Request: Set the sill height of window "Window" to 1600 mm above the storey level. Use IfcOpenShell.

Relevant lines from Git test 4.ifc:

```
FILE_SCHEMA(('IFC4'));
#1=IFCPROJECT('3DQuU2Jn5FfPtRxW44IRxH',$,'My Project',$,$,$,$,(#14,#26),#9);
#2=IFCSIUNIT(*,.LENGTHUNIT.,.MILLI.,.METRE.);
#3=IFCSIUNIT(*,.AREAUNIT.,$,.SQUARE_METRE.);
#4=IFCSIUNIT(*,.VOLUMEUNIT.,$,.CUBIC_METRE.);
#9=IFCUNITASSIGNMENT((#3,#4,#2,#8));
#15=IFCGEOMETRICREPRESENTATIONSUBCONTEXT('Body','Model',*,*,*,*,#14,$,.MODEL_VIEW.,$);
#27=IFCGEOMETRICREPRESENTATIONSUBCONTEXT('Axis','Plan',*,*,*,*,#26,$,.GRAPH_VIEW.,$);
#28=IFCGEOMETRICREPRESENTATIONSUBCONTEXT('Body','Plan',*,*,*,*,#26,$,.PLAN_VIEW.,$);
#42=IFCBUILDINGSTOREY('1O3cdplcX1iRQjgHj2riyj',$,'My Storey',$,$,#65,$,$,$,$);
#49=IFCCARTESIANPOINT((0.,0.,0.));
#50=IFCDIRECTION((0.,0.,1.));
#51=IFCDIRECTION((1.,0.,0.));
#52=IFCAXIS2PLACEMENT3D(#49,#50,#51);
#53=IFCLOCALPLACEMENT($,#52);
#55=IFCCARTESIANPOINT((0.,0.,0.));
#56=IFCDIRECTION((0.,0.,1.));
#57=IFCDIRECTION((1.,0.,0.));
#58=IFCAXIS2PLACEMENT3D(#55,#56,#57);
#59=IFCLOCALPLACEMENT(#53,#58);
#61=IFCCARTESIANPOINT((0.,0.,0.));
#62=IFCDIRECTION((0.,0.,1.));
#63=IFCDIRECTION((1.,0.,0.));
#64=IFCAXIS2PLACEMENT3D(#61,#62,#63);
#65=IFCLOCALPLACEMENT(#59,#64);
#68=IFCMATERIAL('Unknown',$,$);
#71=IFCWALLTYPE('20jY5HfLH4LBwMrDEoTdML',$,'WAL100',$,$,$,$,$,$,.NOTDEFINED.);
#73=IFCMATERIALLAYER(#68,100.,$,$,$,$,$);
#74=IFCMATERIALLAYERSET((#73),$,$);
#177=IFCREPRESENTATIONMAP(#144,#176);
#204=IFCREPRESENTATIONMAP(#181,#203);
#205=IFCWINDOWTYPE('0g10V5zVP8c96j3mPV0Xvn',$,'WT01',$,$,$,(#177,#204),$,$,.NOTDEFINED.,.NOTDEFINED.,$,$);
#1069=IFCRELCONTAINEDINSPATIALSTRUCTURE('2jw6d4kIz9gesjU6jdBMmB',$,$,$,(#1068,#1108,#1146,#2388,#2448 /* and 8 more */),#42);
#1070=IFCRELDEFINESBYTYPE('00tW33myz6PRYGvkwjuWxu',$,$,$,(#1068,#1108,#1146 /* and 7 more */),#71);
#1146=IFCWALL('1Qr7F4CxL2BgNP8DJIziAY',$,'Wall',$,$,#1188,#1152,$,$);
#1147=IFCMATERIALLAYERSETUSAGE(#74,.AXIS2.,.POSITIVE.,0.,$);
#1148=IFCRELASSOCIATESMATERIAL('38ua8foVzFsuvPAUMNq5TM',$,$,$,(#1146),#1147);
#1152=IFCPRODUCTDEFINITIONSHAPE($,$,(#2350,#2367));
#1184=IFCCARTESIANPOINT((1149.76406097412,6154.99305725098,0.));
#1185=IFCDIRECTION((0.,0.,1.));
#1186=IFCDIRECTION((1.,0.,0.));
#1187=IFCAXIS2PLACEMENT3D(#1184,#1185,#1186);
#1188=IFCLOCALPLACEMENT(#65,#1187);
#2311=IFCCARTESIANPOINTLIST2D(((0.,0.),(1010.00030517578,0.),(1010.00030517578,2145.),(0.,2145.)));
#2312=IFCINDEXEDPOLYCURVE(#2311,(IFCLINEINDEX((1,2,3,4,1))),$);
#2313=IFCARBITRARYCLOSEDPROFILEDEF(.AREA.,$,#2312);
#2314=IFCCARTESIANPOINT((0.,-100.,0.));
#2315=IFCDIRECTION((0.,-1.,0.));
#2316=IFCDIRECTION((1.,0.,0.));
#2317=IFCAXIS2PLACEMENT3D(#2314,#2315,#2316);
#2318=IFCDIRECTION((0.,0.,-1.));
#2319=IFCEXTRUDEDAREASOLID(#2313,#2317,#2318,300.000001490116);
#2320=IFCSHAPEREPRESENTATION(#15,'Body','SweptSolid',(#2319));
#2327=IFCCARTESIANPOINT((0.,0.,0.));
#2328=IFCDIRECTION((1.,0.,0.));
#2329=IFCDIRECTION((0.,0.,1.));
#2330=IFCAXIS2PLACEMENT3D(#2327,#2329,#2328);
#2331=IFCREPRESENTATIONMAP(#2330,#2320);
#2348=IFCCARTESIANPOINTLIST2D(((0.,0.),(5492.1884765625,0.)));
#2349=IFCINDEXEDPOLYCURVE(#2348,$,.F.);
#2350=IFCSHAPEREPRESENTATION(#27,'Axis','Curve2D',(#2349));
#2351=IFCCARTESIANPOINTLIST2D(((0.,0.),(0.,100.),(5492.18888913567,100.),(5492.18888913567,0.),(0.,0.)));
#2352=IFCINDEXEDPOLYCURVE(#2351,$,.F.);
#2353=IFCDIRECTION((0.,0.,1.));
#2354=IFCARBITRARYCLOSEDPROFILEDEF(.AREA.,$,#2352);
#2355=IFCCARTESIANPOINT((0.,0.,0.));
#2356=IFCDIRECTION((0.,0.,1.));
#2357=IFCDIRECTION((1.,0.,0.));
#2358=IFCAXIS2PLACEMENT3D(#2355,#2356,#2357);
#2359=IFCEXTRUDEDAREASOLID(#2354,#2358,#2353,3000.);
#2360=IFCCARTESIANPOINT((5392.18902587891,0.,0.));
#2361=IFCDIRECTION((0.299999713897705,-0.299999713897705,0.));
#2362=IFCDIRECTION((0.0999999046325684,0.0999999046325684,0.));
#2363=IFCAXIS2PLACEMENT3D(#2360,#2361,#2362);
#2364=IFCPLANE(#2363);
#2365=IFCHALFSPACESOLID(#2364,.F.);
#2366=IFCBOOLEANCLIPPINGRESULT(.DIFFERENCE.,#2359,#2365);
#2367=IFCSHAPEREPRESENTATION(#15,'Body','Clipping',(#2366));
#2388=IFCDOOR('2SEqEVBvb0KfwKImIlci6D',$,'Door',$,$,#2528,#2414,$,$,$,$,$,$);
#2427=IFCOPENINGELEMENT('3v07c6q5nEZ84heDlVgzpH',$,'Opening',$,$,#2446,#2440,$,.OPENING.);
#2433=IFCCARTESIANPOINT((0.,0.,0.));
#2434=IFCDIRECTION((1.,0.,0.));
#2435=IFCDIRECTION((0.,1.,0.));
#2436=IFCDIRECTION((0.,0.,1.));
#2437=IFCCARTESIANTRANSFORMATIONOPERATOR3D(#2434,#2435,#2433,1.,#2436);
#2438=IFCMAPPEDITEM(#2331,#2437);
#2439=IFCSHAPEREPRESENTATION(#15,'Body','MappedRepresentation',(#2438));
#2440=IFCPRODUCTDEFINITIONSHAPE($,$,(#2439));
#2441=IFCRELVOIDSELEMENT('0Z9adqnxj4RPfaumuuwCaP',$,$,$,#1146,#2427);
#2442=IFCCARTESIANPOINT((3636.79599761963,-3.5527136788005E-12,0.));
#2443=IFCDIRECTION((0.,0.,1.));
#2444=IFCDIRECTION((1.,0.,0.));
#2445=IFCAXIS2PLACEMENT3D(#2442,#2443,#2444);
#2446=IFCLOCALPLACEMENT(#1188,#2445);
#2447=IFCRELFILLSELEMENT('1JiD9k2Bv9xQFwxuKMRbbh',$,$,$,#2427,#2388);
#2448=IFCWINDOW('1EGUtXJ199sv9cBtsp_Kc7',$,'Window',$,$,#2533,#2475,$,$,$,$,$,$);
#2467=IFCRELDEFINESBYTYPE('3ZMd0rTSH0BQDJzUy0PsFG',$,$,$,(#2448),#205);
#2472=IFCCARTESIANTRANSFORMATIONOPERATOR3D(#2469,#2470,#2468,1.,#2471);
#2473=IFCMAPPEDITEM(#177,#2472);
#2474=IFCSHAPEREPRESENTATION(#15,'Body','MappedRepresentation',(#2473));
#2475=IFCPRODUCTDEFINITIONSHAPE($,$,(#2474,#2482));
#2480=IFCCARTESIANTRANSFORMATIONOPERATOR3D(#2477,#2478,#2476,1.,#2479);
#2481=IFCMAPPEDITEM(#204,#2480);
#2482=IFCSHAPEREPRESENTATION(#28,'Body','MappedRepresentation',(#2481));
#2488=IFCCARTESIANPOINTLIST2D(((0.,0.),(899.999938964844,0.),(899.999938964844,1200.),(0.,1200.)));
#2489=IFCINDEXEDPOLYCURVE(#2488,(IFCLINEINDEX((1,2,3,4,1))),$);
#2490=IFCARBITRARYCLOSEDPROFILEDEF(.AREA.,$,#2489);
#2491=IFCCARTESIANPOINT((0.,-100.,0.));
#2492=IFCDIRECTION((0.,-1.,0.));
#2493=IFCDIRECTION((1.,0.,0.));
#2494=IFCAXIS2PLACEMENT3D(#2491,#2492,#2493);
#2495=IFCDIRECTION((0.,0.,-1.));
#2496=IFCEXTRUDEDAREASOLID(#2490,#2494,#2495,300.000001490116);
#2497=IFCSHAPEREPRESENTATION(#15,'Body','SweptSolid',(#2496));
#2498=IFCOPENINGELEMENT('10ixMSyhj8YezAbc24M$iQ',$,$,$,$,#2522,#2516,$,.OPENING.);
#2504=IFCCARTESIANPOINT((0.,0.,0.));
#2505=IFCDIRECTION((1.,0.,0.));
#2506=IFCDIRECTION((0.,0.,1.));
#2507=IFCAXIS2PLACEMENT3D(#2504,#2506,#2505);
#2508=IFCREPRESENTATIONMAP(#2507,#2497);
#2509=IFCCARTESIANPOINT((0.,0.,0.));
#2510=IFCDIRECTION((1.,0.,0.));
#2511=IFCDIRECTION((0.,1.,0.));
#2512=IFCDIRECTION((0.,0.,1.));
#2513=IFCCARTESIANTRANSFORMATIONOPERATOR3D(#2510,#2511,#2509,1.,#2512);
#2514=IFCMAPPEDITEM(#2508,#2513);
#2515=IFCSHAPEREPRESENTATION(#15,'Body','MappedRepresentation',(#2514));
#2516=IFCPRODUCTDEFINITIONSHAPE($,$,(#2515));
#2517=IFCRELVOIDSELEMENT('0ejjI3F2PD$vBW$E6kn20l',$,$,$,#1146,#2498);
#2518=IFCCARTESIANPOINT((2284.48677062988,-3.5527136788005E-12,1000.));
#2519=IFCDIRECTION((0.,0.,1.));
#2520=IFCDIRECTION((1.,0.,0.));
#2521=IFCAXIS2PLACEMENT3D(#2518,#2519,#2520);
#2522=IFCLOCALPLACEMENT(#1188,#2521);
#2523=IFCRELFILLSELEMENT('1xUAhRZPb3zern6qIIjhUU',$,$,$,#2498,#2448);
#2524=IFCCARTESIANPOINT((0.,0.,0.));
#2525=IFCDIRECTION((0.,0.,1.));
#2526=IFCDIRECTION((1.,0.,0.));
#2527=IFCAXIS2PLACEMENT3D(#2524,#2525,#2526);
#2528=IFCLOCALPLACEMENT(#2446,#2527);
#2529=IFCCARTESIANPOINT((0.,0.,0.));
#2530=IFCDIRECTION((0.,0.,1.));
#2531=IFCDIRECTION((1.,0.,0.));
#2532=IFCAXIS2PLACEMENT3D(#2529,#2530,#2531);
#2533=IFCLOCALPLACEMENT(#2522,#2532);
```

```python
import numpy as np
import ifcopenshell
import ifcopenshell.api.geometry
import ifcopenshell.geom
import ifcopenshell.util.element
import ifcopenshell.util.placement
import ifcopenshell.util.shape
import ifcopenshell.util.unit

model = ifcopenshell.open("Git test 4.ifc")
unit_scale = ifcopenshell.util.unit.calculate_unit_scale(model)

window = model.by_guid("1EGUtXJ199sv9cBtsp_Kc7")
opening = window.FillsVoids[0].RelatingOpeningElement
storey = ifcopenshell.util.element.get_container(window, ifc_class="IfcBuildingStorey")
level = ifcopenshell.util.placement.get_local_placement(storey.ObjectPlacement)[2, 3]

# The opening's origin need not be at the sill, so measure its lowest point.
shape = ifcopenshell.geom.create_shape(ifcopenshell.geom.settings(), opening)
bottom = ifcopenshell.util.shape.get_shape_bottom_elevation(shape, shape.geometry) / unit_scale
dz = level + 1600.0 - bottom

shift = np.array([0.0, 0.0, dz])
# The window is placed relative to its opening, so it follows when the opening moves.
matrix = ifcopenshell.util.placement.get_local_placement(opening.ObjectPlacement)
matrix[:3, 3] += shift
ifcopenshell.api.geometry.edit_object_placement(
    model, product=opening, matrix=matrix, is_si=False, should_transform_children=True
)

print(f"moved by {dz * unit_scale:+.3f} m")

model.write("Git test 4-out.ifc")
```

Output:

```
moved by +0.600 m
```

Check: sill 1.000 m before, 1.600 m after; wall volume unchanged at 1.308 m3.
